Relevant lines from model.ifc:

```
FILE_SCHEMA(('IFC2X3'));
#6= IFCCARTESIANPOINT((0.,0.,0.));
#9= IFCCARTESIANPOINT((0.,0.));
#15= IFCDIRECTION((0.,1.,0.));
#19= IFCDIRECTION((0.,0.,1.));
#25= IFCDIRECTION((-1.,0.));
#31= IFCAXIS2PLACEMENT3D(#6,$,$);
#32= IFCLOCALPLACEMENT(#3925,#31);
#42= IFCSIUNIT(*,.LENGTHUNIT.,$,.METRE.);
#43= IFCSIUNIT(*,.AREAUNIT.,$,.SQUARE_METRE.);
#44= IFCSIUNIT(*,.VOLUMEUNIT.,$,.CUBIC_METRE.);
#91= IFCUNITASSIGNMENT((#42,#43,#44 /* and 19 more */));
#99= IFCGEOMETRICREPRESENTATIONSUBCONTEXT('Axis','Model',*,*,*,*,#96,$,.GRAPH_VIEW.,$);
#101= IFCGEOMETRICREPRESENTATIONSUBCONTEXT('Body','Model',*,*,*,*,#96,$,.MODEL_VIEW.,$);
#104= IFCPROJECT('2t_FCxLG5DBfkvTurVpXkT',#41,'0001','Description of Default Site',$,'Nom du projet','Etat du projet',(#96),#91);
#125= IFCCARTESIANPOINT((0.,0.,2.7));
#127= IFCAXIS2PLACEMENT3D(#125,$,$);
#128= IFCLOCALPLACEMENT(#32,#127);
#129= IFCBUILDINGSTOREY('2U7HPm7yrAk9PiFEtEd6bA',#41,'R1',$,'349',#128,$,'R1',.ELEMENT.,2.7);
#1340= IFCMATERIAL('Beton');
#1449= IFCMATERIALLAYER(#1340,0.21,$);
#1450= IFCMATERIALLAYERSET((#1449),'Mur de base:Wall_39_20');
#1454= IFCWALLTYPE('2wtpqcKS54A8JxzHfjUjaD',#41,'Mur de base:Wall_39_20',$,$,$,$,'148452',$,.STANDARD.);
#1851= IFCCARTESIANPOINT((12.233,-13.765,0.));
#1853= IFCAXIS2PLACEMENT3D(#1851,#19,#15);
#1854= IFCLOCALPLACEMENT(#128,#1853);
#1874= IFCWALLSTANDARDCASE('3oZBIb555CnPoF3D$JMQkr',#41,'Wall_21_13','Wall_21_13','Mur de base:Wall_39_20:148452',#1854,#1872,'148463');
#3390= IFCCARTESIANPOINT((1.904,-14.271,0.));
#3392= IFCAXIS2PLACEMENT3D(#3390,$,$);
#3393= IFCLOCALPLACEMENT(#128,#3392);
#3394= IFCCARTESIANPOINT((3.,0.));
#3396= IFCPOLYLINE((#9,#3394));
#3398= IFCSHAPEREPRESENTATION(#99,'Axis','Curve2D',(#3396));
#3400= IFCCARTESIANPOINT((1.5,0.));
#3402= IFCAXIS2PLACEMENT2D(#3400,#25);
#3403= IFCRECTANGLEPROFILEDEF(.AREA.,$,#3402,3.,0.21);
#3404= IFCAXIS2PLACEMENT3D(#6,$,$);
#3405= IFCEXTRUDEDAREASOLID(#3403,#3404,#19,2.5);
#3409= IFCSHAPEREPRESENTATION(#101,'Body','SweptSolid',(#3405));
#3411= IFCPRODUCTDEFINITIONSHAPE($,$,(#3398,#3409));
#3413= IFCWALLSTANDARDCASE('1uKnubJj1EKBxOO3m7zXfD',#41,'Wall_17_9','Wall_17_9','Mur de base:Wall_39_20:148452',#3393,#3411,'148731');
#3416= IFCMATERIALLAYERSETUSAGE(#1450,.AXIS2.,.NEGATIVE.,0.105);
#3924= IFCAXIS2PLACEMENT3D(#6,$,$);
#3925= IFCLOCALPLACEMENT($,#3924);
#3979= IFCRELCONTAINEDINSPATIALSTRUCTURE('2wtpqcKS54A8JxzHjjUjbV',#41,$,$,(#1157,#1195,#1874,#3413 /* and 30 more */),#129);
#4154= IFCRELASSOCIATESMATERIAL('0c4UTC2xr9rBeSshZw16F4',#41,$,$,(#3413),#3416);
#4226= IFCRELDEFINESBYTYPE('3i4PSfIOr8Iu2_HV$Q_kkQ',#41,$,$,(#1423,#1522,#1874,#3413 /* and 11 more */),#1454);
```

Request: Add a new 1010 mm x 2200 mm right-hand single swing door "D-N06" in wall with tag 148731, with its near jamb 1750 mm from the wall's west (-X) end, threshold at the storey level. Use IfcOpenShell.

```python
import numpy as np
import ifcopenshell
import ifcopenshell.api.feature
import ifcopenshell.api.geometry
import ifcopenshell.api.root
import ifcopenshell.api.spatial
import ifcopenshell.api.type
import ifcopenshell.geom
import ifcopenshell.util.element
import ifcopenshell.util.placement
import ifcopenshell.util.representation
import ifcopenshell.util.shape
import ifcopenshell.util.unit

model = ifcopenshell.open("model.ifc")
unit_scale = ifcopenshell.util.unit.calculate_unit_scale(model)
settings = ifcopenshell.geom.settings()


def volume(element):
    """Net volume in cubic metres, openings subtracted."""
    shape = ifcopenshell.geom.create_shape(settings, element)
    return ifcopenshell.util.shape.get_volume(shape.geometry)


wall = model.by_id(3413)
storey = ifcopenshell.util.element.get_container(wall, ifc_class="IfcBuildingStorey")
context = ifcopenshell.util.representation.get_context(model, "Model", "Body", "MODEL_VIEW")
before = volume(wall)

width, height, from_end, sill = 1.01, 2.2, 1.75, 0.0  # metres

# The wall runs along its own X axis, and the end named is its -X end.
wall_shape = ifcopenshell.geom.create_shape(settings, wall)
x, y, z = ifcopenshell.util.shape.get_vertices(wall_shape.geometry).T
start = x.min() + from_end
face, thickness = float(y.min()), float(y.max() - y.min())
wall_matrix = ifcopenshell.util.placement.get_local_placement(wall.ObjectPlacement)
level = ifcopenshell.util.placement.get_local_placement(storey.ObjectPlacement)[2, 3]


def in_wall(x, y):
    """Placement at x, y metres in the wall's axes, at sill height."""
    matrix = wall_matrix.copy()
    matrix[:, 3] = wall_matrix @ np.array([x / unit_scale, y / unit_scale, 0.0, 1.0])
    matrix[2, 3] = level + sill / unit_scale
    return matrix


# Opening: a box that overshoots both wall faces by 50 mm.
opening = ifcopenshell.api.root.create_entity(model, ifc_class="IfcOpeningElement")
box = ifcopenshell.api.geometry.add_wall_representation(
    model, context=context, length=width, height=height, thickness=thickness + 0.1
)
ifcopenshell.api.geometry.assign_representation(model, product=opening, representation=box)
ifcopenshell.api.geometry.edit_object_placement(model, product=opening, matrix=in_wall(start, face - 0.05), is_si=False)
ifcopenshell.api.feature.add_feature(model, feature=opening, element=wall)

door = ifcopenshell.api.root.create_entity(model, ifc_class="IfcDoor", name="D-N06")
door.OverallWidth, door.OverallHeight = width / unit_scale, height / unit_scale
body = ifcopenshell.api.geometry.add_door_representation(
    model,
    context=context,
    overall_width=door.OverallWidth,
    overall_height=door.OverallHeight,
    operation_type="SINGLE_SWING_RIGHT",
    lining_properties={"LiningDepth": thickness / unit_scale, "ThresholdDepth": thickness / unit_scale},
)
ifcopenshell.api.geometry.assign_representation(model, product=door, representation=body)
ifcopenshell.api.spatial.assign_container(model, products=[door], relating_structure=storey)
fills = ifcopenshell.api.feature.add_filling(model, opening=opening, element=door)
fills.OwnerHistory = door.OwnerHistory  # required in IFC2X3

# IFC2X3 keeps the operation on the door style.
style = ifcopenshell.api.root.create_entity(model, ifc_class="IfcDoorStyle", name="D-N06")
style.OperationType, style.ConstructionType = "SINGLE_SWING_RIGHT", "NOTDEFINED"
style.ParameterTakesPrecedence = style.Sizeable = False
ifcopenshell.api.type.assign_type(model, related_objects=[door], relating_type=style)

# The lining spans the wall, so the door starts at the wall face.
ifcopenshell.api.geometry.edit_object_placement(model, product=door, matrix=in_wall(start, face), is_si=False)

after = volume(wall)

print(f"wall volume {before:.3f} -> {after:.3f} m3")

model.write("model_rev.ifc")
```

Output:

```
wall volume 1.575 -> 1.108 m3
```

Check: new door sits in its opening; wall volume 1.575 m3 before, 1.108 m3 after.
